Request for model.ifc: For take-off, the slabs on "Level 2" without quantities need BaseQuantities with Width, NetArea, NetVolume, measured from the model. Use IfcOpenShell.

First a look at what the model holds.

```python
import ifcopenshell
import ifcopenshell.util.element
import ifcopenshell.util.unit

model = ifcopenshell.open("model.ifc")
print(model.schema)
for unit_type in ("LENGTHUNIT", "AREAUNIT", "VOLUMEUNIT"):
    print(unit_type, ifcopenshell.util.unit.calculate_unit_scale(model, unit_type))
storey = next(s for s in model.by_type("IfcBuildingStorey") if s.Name == "Level 2")
slabs = [e for e in ifcopenshell.util.element.get_decomposition(storey) if e.is_a("IfcSlab")]
for e in sorted(slabs, key=lambda e: e.id()):
    print(e.id(), e.is_a(), e.Name, list(ifcopenshell.util.element.get_psets(e, qtos_only=True)), sep=" | ")
```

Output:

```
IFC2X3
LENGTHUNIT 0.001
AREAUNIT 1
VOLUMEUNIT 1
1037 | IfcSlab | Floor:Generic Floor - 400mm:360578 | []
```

```python
import ifcopenshell
import ifcopenshell.api.pset
import ifcopenshell.geom
import ifcopenshell.util.element
import ifcopenshell.util.shape
import ifcopenshell.util.unit

model = ifcopenshell.open("model.ifc")
unit_scale = ifcopenshell.util.unit.calculate_unit_scale(model)
area_scale = ifcopenshell.util.unit.calculate_unit_scale(model, "AREAUNIT")
volume_scale = ifcopenshell.util.unit.calculate_unit_scale(model, "VOLUMEUNIT")
settings = ifcopenshell.geom.settings()

storey = next(s for s in model.by_type("IfcBuildingStorey") if s.Name == "Level 2")
slabs = [e for e in ifcopenshell.util.element.get_decomposition(storey) if e.is_a("IfcSlab")]

for e in sorted(slabs, key=lambda e: e.id()):
    if ifcopenshell.util.element.get_psets(e, qtos_only=True, should_inherit=False):
        continue
    # Geometry comes back in metres, in the element's own axes.
    shape = ifcopenshell.geom.create_shape(settings, e)
    values = {
        "Width": ifcopenshell.util.shape.get_z(shape.geometry) / unit_scale,
        "NetArea": ifcopenshell.util.shape.get_footprint_area(shape.geometry) / area_scale,
        "NetVolume": ifcopenshell.util.shape.get_volume(shape.geometry) / volume_scale,
    }
    qto = ifcopenshell.api.pset.add_qto(model, product=e, name="BaseQuantities")
    ifcopenshell.api.pset.edit_qto(model, qto=qto, properties=values)
    print(e.id(), {k: round(v, 3) for k, v in values.items()})

model.write("model_v2.ifc")
```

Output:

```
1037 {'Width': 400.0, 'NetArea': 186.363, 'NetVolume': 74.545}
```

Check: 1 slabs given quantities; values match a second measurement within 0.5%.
